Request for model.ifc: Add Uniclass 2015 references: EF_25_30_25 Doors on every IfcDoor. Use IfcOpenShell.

First a look at what the model holds.

```python
import ifcopenshell

model = ifcopenshell.open("model.ifc")
print(model.schema)
print("classifications:", [c.Name for c in model.by_type("IfcClassification")])
for ifc_class in ("IfcDoor", "IfcRoof", "IfcStair", "IfcWall", "IfcWindow"):
    print(ifc_class, len(model.by_type(ifc_class)))
```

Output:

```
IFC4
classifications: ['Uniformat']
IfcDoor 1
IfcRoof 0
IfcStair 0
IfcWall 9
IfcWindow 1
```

```python
import ifcopenshell
import ifcopenshell.api.classification

model = ifcopenshell.open("model.ifc")

system = ifcopenshell.api.classification.add_classification(model, classification="Uniclass 2015")

codes = {
    "IfcDoor": ("EF_25_30_25", "Doors"),
}
for ifc_class, (code, name) in codes.items():
    products = model.by_type(ifc_class)
    ifcopenshell.api.classification.add_reference(
        model, products=products, classification=system, identification=code, name=name
    )
    print(code, len(products))

model.write("model_edited.ifc")
```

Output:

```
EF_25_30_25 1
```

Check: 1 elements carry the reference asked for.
